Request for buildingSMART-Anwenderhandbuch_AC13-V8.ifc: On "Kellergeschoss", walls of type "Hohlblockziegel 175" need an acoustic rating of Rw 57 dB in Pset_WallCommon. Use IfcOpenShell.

First a look at what the model holds.

```python
import ifcopenshell
import ifcopenshell.util.element

model = ifcopenshell.open("buildingSMART-Anwenderhandbuch_AC13-V8.ifc")
print(model.schema)
storey = next(s for s in model.by_type("IfcBuildingStorey") if s.Name == "Kellergeschoss")
walls = [e for e in ifcopenshell.util.element.get_decomposition(storey) if e.is_a("IfcWall")]
seen = {}
for e in walls:
    element_type = ifcopenshell.util.element.get_type(e)
    key = (element_type.Name if element_type != e and element_type else None, ifcopenshell.util.element.get_pset(e, "Pset_WallCommon", "AcousticRating"))
    seen[key] = seen.get(key, 0) + 1
for (name, value), count in sorted(seen.items(), key=str):
    print(count, "x", name, "|", value)
```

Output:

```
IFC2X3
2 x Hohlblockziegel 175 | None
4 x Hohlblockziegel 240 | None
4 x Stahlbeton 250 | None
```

```python
import ifcopenshell
import ifcopenshell.api.pset
import ifcopenshell.util.element

model = ifcopenshell.open("buildingSMART-Anwenderhandbuch_AC13-V8.ifc")

storey = next(s for s in model.by_type("IfcBuildingStorey") if s.Name == "Kellergeschoss")
walls = [e for e in ifcopenshell.util.element.get_decomposition(storey) if e.is_a("IfcWall")]

count = 0
for e in walls:
    element_type = ifcopenshell.util.element.get_type(e)
    if element_type in (None, e) or element_type.Name != "Hohlblockziegel 175":
        continue
    # add_pset returns the element's existing set when there is one.
    pset = ifcopenshell.api.pset.add_pset(model, product=e, name="Pset_WallCommon")
    ifcopenshell.api.pset.edit_pset(model, pset=pset, properties={"AcousticRating": "Rw 57 dB"})
    count += 1

print(count, "walls updated")

model.write("buildingSMART-Anwenderhandbuch_AC13-V8_updated.ifc")
```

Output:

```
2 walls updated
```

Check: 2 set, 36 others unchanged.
